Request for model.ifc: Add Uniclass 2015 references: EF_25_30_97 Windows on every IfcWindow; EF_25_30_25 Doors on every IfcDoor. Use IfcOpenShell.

First a look at what the model holds.

```python
import ifcopenshell

model = ifcopenshell.open("model.ifc")
print(model.schema)
print("classifications:", [c.Name for c in model.by_type("IfcClassification")])
for ifc_class in ("IfcDoor", "IfcRoof", "IfcStair", "IfcWall", "IfcWindow"):
    print(ifc_class, len(model.by_type(ifc_class)))
```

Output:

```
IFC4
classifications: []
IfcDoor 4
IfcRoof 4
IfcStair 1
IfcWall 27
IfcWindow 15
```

```python
import ifcopenshell
import ifcopenshell.api.classification

model = ifcopenshell.open("model.ifc")

system = ifcopenshell.api.classification.add_classification(model, classification="Uniclass 2015")

codes = {
    "IfcWindow": ("EF_25_30_97", "Windows"),
    "IfcDoor": ("EF_25_30_25", "Doors"),
}
for ifc_class, (code, name) in codes.items():
    products = model.by_type(ifc_class)
    ifcopenshell.api.classification.add_reference(
        model, products=products, classification=system, identification=code, name=name
    )
    print(code, len(products))

model.write("model_updated.ifc")
```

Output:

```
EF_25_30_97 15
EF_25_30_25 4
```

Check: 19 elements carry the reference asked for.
